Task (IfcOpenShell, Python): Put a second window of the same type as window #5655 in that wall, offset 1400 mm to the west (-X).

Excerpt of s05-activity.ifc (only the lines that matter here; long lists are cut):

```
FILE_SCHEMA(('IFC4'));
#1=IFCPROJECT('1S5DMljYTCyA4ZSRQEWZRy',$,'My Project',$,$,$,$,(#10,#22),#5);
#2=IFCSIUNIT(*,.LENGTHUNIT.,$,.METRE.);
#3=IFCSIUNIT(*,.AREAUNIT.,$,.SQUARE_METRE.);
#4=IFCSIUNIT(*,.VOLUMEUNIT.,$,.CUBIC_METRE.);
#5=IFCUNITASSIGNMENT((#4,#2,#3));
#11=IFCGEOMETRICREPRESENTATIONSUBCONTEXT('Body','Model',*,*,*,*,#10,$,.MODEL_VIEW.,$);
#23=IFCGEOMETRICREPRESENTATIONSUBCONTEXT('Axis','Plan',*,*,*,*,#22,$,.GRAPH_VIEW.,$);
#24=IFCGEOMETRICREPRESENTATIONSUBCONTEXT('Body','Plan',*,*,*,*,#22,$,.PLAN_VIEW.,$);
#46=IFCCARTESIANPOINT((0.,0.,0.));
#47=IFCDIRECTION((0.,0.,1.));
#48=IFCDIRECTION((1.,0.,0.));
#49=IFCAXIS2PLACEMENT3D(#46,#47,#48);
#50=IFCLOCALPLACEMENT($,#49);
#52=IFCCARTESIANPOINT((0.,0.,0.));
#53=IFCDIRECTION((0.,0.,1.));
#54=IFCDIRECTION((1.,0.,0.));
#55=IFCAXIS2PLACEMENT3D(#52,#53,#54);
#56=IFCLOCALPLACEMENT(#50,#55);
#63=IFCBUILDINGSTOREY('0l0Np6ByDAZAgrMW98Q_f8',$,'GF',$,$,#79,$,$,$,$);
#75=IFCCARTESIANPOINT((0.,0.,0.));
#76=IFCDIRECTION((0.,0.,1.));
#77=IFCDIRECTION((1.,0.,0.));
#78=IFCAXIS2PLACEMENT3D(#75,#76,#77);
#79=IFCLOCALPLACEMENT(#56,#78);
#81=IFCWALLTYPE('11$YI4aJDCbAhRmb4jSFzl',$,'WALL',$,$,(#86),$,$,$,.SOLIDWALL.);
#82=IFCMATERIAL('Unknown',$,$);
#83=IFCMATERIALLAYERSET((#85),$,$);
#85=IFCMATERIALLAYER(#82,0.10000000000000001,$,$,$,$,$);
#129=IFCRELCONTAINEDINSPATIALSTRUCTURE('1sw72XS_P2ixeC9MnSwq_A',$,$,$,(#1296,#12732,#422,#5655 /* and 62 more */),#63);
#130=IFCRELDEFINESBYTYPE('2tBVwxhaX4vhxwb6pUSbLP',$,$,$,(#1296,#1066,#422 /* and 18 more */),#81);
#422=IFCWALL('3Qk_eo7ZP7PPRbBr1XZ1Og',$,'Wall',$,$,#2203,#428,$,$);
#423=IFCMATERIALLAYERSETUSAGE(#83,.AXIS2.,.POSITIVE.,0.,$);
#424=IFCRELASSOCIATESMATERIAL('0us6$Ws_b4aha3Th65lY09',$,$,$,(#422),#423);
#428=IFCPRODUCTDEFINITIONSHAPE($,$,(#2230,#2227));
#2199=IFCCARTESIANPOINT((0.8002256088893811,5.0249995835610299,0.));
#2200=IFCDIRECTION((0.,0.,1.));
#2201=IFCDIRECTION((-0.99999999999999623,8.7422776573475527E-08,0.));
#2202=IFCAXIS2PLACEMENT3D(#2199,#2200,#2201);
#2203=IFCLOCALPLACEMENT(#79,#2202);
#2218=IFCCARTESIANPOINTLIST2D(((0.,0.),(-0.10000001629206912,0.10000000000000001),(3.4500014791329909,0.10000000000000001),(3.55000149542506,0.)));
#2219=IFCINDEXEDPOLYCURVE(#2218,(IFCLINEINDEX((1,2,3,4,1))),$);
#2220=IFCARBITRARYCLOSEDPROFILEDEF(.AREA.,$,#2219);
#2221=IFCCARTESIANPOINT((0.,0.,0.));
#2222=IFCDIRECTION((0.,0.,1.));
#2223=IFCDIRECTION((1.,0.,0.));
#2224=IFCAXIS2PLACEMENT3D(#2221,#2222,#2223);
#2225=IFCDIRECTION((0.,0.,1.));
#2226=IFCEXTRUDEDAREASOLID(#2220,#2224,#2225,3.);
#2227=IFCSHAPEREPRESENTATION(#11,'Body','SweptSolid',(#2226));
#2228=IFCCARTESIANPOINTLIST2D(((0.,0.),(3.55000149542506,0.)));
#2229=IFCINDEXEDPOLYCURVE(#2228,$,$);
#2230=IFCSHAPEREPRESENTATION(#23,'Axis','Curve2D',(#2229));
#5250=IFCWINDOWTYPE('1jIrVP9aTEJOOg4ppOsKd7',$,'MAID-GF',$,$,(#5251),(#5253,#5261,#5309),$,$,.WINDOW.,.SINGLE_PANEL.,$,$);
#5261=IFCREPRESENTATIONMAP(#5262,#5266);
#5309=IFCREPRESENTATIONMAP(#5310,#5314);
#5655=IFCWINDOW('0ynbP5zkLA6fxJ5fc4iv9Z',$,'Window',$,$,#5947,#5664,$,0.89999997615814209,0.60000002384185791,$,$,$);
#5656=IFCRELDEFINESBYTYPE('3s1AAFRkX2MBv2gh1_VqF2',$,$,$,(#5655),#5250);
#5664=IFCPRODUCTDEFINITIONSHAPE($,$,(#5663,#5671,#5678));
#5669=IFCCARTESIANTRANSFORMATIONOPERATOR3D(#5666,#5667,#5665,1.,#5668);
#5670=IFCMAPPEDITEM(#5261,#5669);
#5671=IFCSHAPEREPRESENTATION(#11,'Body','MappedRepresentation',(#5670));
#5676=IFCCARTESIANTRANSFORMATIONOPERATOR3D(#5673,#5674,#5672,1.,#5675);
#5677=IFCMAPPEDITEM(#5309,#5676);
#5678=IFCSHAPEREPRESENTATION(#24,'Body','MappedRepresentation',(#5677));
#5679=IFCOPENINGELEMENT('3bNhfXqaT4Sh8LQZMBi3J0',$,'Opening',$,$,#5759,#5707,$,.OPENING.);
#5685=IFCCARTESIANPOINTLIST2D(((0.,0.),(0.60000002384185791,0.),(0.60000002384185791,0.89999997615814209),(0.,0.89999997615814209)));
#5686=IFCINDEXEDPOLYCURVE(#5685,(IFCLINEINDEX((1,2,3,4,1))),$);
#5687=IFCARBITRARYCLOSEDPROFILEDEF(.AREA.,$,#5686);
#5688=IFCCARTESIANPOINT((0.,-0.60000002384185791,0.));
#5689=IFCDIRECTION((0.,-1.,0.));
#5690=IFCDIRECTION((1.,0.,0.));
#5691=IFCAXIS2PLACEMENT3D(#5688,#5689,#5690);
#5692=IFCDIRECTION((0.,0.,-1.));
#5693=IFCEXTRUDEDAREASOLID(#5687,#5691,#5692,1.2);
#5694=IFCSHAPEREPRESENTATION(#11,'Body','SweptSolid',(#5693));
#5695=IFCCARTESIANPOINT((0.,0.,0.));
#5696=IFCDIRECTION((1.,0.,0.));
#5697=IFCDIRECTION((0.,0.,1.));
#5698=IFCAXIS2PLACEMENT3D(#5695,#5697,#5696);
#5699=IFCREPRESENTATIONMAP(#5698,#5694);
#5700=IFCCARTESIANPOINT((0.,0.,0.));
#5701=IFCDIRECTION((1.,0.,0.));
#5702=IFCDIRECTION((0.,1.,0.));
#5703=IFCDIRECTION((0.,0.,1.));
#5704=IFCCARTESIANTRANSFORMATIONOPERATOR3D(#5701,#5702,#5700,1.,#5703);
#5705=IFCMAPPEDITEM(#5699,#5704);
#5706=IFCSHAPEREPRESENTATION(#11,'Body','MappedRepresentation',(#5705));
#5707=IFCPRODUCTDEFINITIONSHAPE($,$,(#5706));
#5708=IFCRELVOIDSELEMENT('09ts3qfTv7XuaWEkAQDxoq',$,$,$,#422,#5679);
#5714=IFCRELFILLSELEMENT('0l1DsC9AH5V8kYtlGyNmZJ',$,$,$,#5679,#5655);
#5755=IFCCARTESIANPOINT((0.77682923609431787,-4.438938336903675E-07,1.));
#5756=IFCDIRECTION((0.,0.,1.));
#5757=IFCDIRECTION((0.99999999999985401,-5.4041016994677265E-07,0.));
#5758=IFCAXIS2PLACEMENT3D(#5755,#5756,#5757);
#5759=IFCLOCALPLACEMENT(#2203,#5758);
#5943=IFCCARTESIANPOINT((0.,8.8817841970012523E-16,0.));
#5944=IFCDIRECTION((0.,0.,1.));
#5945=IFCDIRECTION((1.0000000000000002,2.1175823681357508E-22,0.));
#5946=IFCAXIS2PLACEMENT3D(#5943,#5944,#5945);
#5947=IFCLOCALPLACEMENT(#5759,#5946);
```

```python
import ifcopenshell
import ifcopenshell.api.feature
import ifcopenshell.api.geometry
import ifcopenshell.api.root
import ifcopenshell.geom
import ifcopenshell.util.element
import ifcopenshell.util.placement
import ifcopenshell.util.shape
import ifcopenshell.util.unit

model = ifcopenshell.open("s05-activity.ifc")
unit_scale = ifcopenshell.util.unit.calculate_unit_scale(model)
settings = ifcopenshell.geom.settings()


def volume(element):
    """Net volume in cubic metres, openings subtracted."""
    shape = ifcopenshell.geom.create_shape(settings, element)
    return ifcopenshell.util.shape.get_volume(shape.geometry)


window = model.by_id(5655)
opening = window.FillsVoids[0].RelatingOpeningElement
wall = opening.VoidsElements[0].RelatingBuildingElement
before = volume(wall)
shift = ifcopenshell.util.placement.get_local_placement(wall.ObjectPlacement)[:3, 0] * 1.4 / unit_scale

# copy_class copies the void relationship, type, container and properties, but no geometry.
new_opening = ifcopenshell.api.root.copy_class(model, product=opening)
new_opening.Representation = ifcopenshell.util.element.copy_deep(
    model, opening.Representation, exclude=["IfcGeometricRepresentationContext", "IfcRepresentationMap"]
)
new_window = ifcopenshell.api.root.copy_class(model, product=window)
new_window.Representation = ifcopenshell.util.element.copy_deep(
    model, window.Representation, exclude=["IfcGeometricRepresentationContext", "IfcRepresentationMap"]
)
ifcopenshell.api.feature.add_filling(model, opening=new_opening, element=new_window)

for old, new in ((opening, new_opening), (window, new_window)):
    matrix = ifcopenshell.util.placement.get_local_placement(old.ObjectPlacement)
    matrix[:3, 3] += shift
    ifcopenshell.api.geometry.edit_object_placement(model, product=new, matrix=matrix, is_si=False)

after = volume(wall)

print(f"wall volume {before:.3f} -> {after:.3f} m3")

model.write("s05-activity_edited.ifc")
```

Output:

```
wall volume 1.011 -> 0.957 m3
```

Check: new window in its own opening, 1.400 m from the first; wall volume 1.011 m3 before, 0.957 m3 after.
